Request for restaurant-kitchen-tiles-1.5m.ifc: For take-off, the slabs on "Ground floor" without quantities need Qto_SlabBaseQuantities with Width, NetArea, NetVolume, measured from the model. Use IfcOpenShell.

First a look at what the model holds.

```python
import ifcopenshell
import ifcopenshell.util.element
import ifcopenshell.util.unit

model = ifcopenshell.open("restaurant-kitchen-tiles-1.5m.ifc")
print(model.schema)
for unit_type in ("LENGTHUNIT", "AREAUNIT", "VOLUMEUNIT"):
    print(unit_type, ifcopenshell.util.unit.calculate_unit_scale(model, unit_type))
storey = next(s for s in model.by_type("IfcBuildingStorey") if s.Name == "Ground floor")
slabs = [e for e in ifcopenshell.util.element.get_decomposition(storey) if e.is_a("IfcSlab")]
for e in sorted(slabs, key=lambda e: e.id()):
    print(e.id(), e.is_a(), e.Name, list(ifcopenshell.util.element.get_psets(e, qtos_only=True)), sep=" | ")
```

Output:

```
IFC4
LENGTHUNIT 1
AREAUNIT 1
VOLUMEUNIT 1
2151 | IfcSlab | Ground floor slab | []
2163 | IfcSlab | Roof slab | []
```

```python
import ifcopenshell
import ifcopenshell.api.pset
import ifcopenshell.geom
import ifcopenshell.util.element
import ifcopenshell.util.shape
import ifcopenshell.util.unit

model = ifcopenshell.open("restaurant-kitchen-tiles-1.5m.ifc")
unit_scale = ifcopenshell.util.unit.calculate_unit_scale(model)
area_scale = ifcopenshell.util.unit.calculate_unit_scale(model, "AREAUNIT")
volume_scale = ifcopenshell.util.unit.calculate_unit_scale(model, "VOLUMEUNIT")
settings = ifcopenshell.geom.settings()

storey = next(s for s in model.by_type("IfcBuildingStorey") if s.Name == "Ground floor")
slabs = [e for e in ifcopenshell.util.element.get_decomposition(storey) if e.is_a("IfcSlab")]

for e in sorted(slabs, key=lambda e: e.id()):
    if ifcopenshell.util.element.get_psets(e, qtos_only=True, should_inherit=False):
        continue
    # Geometry comes back in metres, in the element's own axes.
    shape = ifcopenshell.geom.create_shape(settings, e)
    values = {
        "Width": ifcopenshell.util.shape.get_z(shape.geometry) / unit_scale,
        "NetArea": ifcopenshell.util.shape.get_footprint_area(shape.geometry) / area_scale,
        "NetVolume": ifcopenshell.util.shape.get_volume(shape.geometry) / volume_scale,
    }
    qto = ifcopenshell.api.pset.add_qto(model, product=e, name="Qto_SlabBaseQuantities")
    ifcopenshell.api.pset.edit_qto(model, qto=qto, properties=values)
    print(e.id(), {k: round(v, 3) for k, v in values.items()})

model.write("restaurant-kitchen-tiles-1.5m_v2.ifc")
```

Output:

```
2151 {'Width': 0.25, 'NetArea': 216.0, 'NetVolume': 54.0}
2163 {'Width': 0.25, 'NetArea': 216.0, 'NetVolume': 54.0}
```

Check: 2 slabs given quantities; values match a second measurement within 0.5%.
